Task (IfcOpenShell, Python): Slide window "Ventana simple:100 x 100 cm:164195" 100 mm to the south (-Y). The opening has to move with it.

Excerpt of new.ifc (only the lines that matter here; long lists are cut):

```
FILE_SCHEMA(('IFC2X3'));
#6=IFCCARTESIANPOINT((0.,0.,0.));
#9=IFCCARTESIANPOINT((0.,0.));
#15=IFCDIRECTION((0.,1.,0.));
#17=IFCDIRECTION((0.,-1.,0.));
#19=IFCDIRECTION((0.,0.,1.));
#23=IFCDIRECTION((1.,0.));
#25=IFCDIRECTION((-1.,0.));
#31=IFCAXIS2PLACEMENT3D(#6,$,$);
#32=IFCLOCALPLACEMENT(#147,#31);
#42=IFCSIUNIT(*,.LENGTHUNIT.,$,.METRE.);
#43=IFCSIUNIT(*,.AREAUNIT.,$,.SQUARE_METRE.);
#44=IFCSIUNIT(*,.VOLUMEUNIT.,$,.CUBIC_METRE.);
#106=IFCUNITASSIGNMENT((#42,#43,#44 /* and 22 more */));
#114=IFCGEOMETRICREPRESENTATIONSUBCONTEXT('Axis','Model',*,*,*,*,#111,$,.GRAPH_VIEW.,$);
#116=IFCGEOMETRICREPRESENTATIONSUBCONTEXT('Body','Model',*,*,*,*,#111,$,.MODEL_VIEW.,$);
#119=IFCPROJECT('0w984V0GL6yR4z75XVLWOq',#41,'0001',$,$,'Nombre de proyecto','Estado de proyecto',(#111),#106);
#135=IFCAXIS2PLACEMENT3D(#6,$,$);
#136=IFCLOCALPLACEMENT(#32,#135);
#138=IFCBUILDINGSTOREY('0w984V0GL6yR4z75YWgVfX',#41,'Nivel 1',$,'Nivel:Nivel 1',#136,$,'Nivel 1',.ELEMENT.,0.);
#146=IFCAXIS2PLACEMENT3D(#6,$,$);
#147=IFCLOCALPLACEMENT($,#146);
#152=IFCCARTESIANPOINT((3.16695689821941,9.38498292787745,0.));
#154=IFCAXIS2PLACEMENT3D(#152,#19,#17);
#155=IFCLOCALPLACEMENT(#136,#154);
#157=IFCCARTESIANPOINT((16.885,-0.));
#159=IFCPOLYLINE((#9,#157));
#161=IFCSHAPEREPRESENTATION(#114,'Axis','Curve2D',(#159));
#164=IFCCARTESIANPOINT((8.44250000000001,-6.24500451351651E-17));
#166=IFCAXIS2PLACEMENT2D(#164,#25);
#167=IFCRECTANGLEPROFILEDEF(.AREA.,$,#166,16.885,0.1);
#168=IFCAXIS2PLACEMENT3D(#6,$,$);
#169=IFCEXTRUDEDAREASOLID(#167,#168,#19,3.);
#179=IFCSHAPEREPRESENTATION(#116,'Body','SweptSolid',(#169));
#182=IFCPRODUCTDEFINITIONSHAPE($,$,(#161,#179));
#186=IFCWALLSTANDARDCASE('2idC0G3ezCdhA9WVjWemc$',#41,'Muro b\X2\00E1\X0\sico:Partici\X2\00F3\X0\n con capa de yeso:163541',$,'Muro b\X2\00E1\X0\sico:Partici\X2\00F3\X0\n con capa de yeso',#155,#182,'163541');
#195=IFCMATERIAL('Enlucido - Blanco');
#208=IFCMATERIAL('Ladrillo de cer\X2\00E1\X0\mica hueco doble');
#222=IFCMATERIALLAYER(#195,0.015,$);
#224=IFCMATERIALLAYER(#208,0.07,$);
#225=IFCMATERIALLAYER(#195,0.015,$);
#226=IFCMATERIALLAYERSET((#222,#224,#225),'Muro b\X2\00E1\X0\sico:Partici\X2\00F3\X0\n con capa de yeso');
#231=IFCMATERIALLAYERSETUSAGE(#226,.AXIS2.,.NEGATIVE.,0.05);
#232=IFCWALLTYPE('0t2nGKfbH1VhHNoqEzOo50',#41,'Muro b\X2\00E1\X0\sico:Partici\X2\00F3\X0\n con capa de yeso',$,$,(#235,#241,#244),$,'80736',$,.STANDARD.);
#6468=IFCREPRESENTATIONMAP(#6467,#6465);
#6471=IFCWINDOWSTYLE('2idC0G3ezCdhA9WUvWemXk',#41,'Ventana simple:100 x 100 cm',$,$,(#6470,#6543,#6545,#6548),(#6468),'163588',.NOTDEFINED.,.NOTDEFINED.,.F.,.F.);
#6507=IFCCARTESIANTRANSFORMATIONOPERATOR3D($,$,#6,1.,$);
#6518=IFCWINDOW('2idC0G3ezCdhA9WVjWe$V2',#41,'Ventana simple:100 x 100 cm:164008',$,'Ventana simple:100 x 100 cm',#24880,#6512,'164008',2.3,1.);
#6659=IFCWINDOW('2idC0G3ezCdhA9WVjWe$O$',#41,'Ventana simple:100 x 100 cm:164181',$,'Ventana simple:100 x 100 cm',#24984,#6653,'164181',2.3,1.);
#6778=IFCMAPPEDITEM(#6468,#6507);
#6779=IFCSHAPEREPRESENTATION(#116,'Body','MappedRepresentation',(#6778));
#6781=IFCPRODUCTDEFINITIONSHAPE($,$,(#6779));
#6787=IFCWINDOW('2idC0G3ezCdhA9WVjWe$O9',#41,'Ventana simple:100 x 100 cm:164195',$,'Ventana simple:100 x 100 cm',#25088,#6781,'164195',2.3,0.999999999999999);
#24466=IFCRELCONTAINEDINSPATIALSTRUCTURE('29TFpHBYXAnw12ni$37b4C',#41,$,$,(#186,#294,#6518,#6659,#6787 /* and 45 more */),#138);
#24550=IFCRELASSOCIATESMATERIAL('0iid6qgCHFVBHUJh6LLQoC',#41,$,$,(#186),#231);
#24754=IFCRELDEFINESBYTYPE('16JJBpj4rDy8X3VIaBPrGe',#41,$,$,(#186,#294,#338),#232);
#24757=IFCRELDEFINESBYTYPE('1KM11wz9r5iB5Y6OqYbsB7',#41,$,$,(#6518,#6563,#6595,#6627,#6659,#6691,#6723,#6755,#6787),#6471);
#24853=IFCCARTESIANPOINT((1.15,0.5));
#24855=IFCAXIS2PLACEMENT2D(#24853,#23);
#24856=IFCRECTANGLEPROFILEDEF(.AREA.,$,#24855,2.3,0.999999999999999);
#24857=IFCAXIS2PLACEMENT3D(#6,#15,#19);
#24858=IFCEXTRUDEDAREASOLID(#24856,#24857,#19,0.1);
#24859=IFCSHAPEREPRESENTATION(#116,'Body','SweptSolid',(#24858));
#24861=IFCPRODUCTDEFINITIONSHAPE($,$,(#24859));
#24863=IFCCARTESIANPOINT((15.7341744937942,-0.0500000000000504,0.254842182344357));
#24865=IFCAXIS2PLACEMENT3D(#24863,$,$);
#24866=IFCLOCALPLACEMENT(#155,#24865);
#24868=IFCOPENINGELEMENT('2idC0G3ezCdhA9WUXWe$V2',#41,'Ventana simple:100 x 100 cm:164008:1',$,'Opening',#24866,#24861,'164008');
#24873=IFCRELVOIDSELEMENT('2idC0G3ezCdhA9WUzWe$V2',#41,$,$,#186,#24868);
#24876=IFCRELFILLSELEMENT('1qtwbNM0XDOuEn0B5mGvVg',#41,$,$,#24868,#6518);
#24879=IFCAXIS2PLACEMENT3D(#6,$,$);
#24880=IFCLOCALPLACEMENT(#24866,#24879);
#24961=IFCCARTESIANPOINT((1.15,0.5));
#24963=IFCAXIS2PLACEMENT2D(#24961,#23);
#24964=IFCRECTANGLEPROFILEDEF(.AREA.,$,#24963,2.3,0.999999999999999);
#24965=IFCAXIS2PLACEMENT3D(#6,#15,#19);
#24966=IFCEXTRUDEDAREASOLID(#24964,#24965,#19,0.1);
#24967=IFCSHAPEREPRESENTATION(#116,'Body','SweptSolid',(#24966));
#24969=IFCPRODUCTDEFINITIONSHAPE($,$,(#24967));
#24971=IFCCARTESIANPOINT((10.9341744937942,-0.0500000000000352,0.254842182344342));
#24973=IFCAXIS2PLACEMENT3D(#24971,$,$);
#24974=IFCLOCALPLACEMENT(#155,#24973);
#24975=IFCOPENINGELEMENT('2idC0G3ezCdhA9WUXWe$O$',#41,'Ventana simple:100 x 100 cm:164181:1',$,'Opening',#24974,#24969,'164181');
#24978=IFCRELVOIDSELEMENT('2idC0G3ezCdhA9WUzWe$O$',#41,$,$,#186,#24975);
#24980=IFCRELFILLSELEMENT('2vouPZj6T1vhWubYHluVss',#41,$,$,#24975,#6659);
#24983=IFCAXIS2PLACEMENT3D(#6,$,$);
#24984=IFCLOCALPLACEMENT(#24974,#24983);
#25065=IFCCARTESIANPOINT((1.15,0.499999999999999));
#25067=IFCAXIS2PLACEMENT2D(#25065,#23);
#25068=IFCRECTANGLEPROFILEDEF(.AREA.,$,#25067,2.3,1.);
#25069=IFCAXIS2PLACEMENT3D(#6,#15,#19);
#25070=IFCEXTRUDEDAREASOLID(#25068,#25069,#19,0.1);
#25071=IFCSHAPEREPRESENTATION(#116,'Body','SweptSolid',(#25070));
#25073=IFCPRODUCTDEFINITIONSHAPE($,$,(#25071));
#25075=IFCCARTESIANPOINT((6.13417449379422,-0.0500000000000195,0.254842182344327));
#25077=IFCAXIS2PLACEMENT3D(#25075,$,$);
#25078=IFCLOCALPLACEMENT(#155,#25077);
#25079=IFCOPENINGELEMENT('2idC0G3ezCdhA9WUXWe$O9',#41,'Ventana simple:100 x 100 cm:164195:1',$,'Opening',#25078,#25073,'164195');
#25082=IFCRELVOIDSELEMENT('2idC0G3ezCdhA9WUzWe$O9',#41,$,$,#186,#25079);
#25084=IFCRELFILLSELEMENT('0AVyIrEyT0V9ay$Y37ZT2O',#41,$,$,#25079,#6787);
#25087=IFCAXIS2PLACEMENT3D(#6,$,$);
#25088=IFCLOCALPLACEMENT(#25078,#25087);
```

```python
import ifcopenshell
import ifcopenshell.api.geometry
import ifcopenshell.util.placement
import ifcopenshell.util.unit

model = ifcopenshell.open("new.ifc")
unit_scale = ifcopenshell.util.unit.calculate_unit_scale(model)

window = model.by_guid("2idC0G3ezCdhA9WVjWe$O9")
opening = window.FillsVoids[0].RelatingOpeningElement
wall = opening.VoidsElements[0].RelatingBuildingElement

wall_matrix = ifcopenshell.util.placement.get_local_placement(wall.ObjectPlacement)
shift = wall_matrix[:3, 0] * 0.1 / unit_scale
before = ifcopenshell.util.placement.get_local_placement(window.ObjectPlacement)[:3, 3].copy()

# The window is placed relative to its opening, so it follows when the opening moves.
matrix = ifcopenshell.util.placement.get_local_placement(opening.ObjectPlacement)
matrix[:3, 3] += shift
ifcopenshell.api.geometry.edit_object_placement(
    model, product=opening, matrix=matrix, is_si=False, should_transform_children=True
)

after = ifcopenshell.util.placement.get_local_placement(window.ObjectPlacement)[:3, 3]
print("window moved by", (after - before).round(3) + 0.0)

model.write("new_edited.ifc")
```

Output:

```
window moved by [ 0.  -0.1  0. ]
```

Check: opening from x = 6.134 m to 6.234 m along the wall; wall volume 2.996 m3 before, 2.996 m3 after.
